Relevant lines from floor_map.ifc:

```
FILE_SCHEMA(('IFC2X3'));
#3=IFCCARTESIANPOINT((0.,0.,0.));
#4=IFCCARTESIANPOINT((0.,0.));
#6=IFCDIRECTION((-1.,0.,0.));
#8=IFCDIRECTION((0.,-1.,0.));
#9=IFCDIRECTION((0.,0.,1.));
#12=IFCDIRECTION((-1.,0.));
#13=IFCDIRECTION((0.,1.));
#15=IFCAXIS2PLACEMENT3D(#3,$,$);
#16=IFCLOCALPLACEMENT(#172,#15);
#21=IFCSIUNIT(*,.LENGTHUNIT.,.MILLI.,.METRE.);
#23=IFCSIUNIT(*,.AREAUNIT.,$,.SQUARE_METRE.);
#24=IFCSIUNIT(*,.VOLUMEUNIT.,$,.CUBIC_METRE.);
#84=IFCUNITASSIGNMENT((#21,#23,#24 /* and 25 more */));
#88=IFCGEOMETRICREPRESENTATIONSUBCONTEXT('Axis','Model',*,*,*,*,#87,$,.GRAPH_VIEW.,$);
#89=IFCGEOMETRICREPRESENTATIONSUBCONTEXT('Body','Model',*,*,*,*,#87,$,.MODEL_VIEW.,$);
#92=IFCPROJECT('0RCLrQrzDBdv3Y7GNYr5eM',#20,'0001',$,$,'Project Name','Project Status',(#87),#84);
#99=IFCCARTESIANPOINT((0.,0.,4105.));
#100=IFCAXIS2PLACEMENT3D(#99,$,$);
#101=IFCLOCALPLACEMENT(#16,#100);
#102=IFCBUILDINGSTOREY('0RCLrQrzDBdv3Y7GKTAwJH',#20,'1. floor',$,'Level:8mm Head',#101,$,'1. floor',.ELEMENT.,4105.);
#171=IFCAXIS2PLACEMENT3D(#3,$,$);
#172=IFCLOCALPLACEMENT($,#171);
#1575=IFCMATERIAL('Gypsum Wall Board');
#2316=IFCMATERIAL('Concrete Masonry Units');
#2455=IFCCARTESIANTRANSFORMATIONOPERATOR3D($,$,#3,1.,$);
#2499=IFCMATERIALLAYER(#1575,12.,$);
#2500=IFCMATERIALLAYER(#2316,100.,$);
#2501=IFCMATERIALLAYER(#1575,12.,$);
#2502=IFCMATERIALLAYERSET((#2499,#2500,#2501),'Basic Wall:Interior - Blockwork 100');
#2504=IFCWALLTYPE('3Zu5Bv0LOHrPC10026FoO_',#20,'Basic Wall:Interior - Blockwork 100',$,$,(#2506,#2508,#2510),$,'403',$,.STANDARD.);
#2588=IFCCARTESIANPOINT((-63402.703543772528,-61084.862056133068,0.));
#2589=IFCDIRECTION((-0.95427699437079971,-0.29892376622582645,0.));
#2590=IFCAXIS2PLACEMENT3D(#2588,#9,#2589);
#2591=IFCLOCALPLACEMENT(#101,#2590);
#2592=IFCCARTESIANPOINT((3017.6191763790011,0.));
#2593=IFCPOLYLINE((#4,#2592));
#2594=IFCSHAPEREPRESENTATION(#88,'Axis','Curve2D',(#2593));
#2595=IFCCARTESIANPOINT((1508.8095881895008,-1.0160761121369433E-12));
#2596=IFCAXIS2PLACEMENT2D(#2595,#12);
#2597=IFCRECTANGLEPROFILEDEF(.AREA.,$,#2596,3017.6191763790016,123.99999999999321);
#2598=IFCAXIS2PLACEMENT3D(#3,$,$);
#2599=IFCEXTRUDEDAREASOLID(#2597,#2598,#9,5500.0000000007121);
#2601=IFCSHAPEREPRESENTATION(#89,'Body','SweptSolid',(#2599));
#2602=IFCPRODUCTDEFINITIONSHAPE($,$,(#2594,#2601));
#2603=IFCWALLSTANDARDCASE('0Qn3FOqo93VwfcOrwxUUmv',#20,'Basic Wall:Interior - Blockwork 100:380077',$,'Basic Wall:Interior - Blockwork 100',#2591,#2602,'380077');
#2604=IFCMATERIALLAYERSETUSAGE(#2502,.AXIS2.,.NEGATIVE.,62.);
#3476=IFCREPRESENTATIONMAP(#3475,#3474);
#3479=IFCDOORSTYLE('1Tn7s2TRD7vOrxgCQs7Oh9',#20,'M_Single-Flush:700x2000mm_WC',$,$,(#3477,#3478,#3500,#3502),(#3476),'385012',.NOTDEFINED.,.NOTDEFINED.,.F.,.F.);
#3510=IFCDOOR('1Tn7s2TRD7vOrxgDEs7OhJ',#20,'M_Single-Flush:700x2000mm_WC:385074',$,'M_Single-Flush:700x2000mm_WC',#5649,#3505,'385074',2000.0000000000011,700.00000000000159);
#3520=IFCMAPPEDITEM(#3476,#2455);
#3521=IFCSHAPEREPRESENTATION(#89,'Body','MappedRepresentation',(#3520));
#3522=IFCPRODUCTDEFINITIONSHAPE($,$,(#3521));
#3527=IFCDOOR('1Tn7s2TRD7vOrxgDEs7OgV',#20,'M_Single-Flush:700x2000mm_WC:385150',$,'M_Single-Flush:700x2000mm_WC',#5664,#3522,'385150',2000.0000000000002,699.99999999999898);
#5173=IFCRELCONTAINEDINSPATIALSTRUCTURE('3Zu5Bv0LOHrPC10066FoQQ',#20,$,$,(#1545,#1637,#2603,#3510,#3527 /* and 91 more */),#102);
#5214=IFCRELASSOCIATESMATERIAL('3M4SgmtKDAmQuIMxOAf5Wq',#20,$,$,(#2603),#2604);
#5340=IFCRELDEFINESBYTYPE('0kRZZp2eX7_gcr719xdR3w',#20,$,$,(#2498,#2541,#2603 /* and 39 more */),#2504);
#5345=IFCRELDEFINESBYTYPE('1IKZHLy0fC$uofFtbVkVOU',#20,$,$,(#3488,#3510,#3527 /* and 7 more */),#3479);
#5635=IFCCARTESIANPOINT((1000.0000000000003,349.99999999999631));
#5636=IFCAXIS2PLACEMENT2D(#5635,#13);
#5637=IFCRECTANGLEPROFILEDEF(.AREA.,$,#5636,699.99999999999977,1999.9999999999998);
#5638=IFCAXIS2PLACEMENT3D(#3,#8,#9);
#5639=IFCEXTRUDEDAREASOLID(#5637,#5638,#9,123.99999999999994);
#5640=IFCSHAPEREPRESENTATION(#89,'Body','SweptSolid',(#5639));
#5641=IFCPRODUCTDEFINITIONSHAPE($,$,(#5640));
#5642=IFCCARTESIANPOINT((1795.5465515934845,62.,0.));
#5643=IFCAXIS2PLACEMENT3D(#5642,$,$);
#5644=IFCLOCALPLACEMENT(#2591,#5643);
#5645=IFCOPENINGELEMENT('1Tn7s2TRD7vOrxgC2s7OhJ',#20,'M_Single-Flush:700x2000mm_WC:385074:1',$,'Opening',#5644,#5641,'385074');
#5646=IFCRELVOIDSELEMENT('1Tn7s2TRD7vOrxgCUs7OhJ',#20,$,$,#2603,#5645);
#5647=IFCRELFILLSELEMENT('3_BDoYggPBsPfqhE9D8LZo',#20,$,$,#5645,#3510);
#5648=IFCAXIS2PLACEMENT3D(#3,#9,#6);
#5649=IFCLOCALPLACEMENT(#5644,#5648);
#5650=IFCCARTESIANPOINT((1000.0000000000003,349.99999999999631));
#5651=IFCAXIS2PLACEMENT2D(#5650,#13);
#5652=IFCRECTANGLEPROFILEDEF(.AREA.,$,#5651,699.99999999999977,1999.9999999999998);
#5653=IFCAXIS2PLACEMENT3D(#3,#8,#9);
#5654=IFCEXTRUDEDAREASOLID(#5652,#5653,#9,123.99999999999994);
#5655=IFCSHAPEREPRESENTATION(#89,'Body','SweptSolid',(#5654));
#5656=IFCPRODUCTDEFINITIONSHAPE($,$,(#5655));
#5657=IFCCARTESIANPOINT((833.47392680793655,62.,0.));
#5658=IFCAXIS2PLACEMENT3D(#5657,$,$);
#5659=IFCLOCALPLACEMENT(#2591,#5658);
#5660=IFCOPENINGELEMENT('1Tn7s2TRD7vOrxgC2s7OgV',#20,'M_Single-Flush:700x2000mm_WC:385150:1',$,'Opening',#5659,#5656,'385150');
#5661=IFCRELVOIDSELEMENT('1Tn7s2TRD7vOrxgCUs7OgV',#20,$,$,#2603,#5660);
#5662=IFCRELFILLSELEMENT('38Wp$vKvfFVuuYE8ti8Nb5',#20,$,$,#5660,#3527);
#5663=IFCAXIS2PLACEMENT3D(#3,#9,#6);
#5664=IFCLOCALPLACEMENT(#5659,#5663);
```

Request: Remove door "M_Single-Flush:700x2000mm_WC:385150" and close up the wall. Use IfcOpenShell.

```python
import ifcopenshell
import ifcopenshell.api.feature
import ifcopenshell.api.root
import ifcopenshell.geom
import ifcopenshell.util.shape

model = ifcopenshell.open("floor_map.ifc")
settings = ifcopenshell.geom.settings()


def volume(element):
    """Net volume in cubic metres, openings subtracted."""
    shape = ifcopenshell.geom.create_shape(settings, element)
    return ifcopenshell.util.shape.get_volume(shape.geometry)


door = model.by_id(3527)
opening = door.FillsVoids[0].RelatingOpeningElement
wall = opening.VoidsElements[0].RelatingBuildingElement
before = volume(wall)

ifcopenshell.api.root.remove_product(model, product=door)
ifcopenshell.api.feature.remove_feature(model, feature=opening)

after = volume(wall)

print(f"wall volume {before:.3f} -> {after:.3f} m3")

model.write("floor_map_rev.ifc")
```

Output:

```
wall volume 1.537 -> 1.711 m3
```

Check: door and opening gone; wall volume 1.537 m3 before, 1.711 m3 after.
